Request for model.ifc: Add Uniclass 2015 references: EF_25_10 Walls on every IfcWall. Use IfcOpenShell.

First a look at what the model holds.

```python
import ifcopenshell

model = ifcopenshell.open("model.ifc")
print(model.schema)
print("classifications:", [c.Name for c in model.by_type("IfcClassification")])
for ifc_class in ("IfcDoor", "IfcRoof", "IfcStair", "IfcWall", "IfcWindow"):
    print(ifc_class, len(model.by_type(ifc_class)))
```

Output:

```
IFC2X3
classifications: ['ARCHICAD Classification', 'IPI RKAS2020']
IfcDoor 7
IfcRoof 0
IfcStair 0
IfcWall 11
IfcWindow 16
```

```python
import ifcopenshell
import ifcopenshell.api.classification

model = ifcopenshell.open("model.ifc")

# IFC2X3 requires Source and Edition and has no link from the project to the system.
system = model.create_entity("IfcClassification", Source="NBS", Edition="2015", Name="Uniclass 2015")

codes = {
    "IfcWall": ("EF_25_10", "Walls"),
}
for ifc_class, (code, name) in codes.items():
    products = model.by_type(ifc_class)
    ifcopenshell.api.classification.add_reference(
        model, products=products, classification=system, identification=code, name=name
    )
    print(code, len(products))

model.write("model_edited.ifc")
```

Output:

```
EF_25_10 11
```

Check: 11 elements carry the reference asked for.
